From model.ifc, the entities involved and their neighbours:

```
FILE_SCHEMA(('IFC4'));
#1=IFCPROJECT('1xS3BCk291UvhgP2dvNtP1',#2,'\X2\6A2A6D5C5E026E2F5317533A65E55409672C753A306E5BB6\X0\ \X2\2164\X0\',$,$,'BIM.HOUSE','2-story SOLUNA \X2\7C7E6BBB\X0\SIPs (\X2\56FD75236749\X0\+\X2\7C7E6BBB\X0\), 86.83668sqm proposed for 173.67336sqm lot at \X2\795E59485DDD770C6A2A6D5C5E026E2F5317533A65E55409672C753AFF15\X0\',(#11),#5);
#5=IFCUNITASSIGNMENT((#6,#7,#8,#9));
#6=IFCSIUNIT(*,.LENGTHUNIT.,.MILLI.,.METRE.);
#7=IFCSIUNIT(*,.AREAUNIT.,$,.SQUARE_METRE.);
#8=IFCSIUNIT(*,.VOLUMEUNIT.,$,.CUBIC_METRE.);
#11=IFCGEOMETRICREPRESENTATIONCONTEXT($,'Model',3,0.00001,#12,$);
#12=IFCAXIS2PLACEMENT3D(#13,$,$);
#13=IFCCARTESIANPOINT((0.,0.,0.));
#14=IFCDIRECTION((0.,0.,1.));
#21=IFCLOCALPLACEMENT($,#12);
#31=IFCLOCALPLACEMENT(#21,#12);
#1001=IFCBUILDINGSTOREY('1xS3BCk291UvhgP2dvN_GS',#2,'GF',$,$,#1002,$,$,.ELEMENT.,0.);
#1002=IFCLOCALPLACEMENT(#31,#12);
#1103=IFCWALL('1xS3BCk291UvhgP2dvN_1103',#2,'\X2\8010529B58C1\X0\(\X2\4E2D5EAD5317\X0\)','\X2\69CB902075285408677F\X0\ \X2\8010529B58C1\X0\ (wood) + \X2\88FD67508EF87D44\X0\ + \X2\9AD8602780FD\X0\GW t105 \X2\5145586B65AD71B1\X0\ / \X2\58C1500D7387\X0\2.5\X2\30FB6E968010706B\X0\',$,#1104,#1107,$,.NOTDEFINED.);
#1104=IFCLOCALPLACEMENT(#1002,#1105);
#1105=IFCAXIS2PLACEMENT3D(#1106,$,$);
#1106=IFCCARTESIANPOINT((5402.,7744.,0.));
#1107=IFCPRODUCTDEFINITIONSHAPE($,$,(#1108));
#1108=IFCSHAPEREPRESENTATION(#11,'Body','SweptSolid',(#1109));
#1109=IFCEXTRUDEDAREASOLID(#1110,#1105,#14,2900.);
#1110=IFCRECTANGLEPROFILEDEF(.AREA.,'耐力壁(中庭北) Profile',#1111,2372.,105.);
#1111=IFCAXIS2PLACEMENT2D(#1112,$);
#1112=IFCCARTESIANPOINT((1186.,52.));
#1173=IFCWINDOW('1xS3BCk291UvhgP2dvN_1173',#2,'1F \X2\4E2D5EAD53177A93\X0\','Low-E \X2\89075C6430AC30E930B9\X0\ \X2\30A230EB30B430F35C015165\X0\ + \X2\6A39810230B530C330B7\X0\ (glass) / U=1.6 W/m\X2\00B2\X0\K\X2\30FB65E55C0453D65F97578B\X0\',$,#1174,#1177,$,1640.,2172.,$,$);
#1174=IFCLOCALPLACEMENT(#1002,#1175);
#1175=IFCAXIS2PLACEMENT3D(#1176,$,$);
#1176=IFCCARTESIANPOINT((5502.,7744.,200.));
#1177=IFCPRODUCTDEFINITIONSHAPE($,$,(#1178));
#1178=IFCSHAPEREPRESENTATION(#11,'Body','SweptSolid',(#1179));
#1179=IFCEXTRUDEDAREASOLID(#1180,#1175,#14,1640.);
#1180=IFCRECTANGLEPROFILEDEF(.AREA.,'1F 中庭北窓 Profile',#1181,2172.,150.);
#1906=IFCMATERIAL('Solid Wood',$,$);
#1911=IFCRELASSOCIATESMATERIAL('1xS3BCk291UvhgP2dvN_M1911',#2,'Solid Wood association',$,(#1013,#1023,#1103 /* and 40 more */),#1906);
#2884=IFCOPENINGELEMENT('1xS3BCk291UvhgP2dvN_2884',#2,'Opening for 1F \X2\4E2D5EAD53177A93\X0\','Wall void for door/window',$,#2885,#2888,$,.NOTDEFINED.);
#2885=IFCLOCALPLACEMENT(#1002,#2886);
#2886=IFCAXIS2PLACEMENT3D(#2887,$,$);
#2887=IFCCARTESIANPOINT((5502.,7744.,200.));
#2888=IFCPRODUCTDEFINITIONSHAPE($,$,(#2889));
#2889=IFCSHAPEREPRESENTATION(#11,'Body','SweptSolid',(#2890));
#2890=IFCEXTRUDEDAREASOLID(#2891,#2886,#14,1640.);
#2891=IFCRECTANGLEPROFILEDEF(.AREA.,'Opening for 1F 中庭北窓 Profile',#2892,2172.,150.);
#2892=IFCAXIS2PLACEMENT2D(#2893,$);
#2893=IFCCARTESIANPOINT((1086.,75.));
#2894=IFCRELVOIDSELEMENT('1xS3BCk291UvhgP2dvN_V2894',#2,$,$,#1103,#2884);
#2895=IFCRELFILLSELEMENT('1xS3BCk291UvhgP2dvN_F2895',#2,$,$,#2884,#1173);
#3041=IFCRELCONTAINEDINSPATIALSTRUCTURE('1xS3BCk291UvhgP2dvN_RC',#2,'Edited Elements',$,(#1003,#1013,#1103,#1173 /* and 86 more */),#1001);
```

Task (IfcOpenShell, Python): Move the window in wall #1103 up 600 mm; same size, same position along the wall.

```python
import numpy as np
import ifcopenshell
import ifcopenshell.api.geometry
import ifcopenshell.util.placement
import ifcopenshell.util.unit

model = ifcopenshell.open("model.ifc")
unit_scale = ifcopenshell.util.unit.calculate_unit_scale(model)

window = model.by_id(1173)
opening = window.FillsVoids[0].RelatingOpeningElement
dz = 0.6 / unit_scale

shift = np.array([0.0, 0.0, dz])
# The window is not placed relative to its opening, so move both.
for product in (opening, window):
    matrix = ifcopenshell.util.placement.get_local_placement(product.ObjectPlacement)
    matrix[:3, 3] += shift
    ifcopenshell.api.geometry.edit_object_placement(model, product=product, matrix=matrix, is_si=False)

print(f"moved by {dz * unit_scale:+.3f} m")

model.write("model_v2.ifc")
```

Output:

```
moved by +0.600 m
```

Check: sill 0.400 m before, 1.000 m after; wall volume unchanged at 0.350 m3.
